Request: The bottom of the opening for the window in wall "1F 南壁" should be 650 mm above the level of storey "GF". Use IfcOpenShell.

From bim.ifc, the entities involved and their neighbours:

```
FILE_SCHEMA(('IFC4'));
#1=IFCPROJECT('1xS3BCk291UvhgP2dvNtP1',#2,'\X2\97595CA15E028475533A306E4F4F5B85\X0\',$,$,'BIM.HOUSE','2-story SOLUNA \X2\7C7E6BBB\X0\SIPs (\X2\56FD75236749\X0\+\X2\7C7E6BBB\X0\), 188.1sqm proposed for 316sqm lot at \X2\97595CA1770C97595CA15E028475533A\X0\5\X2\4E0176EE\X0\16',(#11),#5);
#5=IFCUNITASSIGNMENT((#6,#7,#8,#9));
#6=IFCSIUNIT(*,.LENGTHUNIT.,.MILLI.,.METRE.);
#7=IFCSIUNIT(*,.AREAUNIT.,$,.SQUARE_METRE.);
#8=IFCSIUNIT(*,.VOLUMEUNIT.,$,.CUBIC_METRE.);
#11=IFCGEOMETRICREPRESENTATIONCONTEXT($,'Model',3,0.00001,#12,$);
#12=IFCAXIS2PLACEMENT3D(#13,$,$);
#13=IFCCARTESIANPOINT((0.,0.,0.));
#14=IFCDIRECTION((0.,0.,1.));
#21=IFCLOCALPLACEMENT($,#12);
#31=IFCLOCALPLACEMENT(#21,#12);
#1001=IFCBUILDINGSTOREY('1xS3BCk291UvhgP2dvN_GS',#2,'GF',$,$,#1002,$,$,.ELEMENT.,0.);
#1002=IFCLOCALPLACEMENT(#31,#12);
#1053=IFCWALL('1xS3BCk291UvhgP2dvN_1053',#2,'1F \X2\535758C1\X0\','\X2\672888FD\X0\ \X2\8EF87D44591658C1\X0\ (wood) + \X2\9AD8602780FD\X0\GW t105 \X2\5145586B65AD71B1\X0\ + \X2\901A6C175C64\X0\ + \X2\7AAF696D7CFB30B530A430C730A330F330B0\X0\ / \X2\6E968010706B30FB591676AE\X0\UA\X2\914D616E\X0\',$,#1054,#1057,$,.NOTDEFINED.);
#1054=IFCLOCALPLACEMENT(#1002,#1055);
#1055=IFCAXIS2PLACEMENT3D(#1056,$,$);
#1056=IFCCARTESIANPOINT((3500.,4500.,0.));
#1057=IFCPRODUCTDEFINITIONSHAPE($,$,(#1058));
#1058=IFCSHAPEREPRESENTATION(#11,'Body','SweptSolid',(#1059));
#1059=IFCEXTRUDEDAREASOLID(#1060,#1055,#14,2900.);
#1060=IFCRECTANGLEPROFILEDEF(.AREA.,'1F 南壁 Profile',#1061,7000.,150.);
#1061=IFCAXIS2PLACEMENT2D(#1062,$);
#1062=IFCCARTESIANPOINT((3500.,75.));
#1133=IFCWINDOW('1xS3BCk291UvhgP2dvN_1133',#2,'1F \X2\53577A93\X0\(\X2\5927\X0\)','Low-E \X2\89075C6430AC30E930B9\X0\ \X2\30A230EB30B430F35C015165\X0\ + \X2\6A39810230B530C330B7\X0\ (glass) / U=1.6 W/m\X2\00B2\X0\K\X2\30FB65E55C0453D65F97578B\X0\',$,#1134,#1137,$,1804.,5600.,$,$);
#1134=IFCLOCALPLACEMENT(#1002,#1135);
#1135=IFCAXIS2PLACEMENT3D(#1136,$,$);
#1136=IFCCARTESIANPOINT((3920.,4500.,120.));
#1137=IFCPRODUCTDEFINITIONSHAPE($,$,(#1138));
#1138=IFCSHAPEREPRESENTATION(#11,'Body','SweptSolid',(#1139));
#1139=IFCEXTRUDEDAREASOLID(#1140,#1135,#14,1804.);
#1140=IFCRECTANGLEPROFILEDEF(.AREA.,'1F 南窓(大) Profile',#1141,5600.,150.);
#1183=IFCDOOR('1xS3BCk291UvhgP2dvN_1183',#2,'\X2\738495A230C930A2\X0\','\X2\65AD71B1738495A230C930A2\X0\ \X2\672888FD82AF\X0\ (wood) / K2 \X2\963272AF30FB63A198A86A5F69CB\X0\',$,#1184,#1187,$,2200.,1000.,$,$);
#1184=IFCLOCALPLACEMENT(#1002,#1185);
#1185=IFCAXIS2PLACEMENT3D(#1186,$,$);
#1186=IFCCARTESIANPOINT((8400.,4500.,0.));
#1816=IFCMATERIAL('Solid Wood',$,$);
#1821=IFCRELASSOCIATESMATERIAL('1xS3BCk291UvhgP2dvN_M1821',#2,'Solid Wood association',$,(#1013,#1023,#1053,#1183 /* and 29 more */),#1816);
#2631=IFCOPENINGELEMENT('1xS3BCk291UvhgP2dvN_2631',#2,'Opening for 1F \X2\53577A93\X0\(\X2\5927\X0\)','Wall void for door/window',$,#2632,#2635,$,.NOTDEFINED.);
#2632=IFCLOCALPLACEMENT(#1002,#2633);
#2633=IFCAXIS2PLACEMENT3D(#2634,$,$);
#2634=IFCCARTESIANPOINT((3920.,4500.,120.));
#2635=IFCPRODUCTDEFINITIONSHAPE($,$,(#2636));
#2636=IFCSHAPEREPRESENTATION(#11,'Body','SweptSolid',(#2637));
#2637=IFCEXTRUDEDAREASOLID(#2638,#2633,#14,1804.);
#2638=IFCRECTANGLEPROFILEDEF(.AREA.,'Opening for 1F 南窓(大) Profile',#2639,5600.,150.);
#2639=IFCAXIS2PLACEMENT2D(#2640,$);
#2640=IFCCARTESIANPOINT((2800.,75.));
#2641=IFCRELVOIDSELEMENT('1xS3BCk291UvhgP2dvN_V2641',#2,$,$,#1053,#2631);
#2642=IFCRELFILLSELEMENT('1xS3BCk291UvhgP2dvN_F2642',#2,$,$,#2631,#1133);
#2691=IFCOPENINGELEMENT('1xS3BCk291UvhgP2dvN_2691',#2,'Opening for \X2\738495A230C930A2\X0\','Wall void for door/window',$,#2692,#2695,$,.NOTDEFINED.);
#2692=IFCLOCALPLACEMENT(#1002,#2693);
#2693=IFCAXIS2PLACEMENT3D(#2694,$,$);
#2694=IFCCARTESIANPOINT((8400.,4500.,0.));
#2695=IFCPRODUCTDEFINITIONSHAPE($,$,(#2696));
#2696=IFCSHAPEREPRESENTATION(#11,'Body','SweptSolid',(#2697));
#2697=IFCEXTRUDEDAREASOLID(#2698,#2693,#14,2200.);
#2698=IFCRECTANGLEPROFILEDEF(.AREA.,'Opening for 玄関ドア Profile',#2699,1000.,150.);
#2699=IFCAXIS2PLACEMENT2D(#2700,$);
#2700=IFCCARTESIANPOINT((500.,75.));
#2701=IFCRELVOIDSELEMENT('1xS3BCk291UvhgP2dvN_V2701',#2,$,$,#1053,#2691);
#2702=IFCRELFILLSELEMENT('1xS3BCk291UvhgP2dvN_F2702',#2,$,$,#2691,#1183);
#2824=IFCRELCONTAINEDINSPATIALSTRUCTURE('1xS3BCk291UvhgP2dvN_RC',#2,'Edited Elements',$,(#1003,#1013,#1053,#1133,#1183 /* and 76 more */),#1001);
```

```python
import numpy as np
import ifcopenshell
import ifcopenshell.api.geometry
import ifcopenshell.geom
import ifcopenshell.util.element
import ifcopenshell.util.placement
import ifcopenshell.util.shape
import ifcopenshell.util.unit

model = ifcopenshell.open("bim.ifc")
unit_scale = ifcopenshell.util.unit.calculate_unit_scale(model)

window = model.by_id(1133)
opening = window.FillsVoids[0].RelatingOpeningElement
storey = ifcopenshell.util.element.get_container(window, ifc_class="IfcBuildingStorey")
level = ifcopenshell.util.placement.get_local_placement(storey.ObjectPlacement)[2, 3]

# The opening's origin need not be at the sill, so measure its lowest point.
shape = ifcopenshell.geom.create_shape(ifcopenshell.geom.settings(), opening)
bottom = ifcopenshell.util.shape.get_shape_bottom_elevation(shape, shape.geometry) / unit_scale
dz = level + 650.0 - bottom

shift = np.array([0.0, 0.0, dz])
# The window is not placed relative to its opening, so move both.
for product in (opening, window):
    matrix = ifcopenshell.util.placement.get_local_placement(product.ObjectPlacement)
    matrix[:3, 3] += shift
    ifcopenshell.api.geometry.edit_object_placement(model, product=product, matrix=matrix, is_si=False)

print(f"moved by {dz * unit_scale:+.3f} m")

model.write("bim_edited.ifc")
```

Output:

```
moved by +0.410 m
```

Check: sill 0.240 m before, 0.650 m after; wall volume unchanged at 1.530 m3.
